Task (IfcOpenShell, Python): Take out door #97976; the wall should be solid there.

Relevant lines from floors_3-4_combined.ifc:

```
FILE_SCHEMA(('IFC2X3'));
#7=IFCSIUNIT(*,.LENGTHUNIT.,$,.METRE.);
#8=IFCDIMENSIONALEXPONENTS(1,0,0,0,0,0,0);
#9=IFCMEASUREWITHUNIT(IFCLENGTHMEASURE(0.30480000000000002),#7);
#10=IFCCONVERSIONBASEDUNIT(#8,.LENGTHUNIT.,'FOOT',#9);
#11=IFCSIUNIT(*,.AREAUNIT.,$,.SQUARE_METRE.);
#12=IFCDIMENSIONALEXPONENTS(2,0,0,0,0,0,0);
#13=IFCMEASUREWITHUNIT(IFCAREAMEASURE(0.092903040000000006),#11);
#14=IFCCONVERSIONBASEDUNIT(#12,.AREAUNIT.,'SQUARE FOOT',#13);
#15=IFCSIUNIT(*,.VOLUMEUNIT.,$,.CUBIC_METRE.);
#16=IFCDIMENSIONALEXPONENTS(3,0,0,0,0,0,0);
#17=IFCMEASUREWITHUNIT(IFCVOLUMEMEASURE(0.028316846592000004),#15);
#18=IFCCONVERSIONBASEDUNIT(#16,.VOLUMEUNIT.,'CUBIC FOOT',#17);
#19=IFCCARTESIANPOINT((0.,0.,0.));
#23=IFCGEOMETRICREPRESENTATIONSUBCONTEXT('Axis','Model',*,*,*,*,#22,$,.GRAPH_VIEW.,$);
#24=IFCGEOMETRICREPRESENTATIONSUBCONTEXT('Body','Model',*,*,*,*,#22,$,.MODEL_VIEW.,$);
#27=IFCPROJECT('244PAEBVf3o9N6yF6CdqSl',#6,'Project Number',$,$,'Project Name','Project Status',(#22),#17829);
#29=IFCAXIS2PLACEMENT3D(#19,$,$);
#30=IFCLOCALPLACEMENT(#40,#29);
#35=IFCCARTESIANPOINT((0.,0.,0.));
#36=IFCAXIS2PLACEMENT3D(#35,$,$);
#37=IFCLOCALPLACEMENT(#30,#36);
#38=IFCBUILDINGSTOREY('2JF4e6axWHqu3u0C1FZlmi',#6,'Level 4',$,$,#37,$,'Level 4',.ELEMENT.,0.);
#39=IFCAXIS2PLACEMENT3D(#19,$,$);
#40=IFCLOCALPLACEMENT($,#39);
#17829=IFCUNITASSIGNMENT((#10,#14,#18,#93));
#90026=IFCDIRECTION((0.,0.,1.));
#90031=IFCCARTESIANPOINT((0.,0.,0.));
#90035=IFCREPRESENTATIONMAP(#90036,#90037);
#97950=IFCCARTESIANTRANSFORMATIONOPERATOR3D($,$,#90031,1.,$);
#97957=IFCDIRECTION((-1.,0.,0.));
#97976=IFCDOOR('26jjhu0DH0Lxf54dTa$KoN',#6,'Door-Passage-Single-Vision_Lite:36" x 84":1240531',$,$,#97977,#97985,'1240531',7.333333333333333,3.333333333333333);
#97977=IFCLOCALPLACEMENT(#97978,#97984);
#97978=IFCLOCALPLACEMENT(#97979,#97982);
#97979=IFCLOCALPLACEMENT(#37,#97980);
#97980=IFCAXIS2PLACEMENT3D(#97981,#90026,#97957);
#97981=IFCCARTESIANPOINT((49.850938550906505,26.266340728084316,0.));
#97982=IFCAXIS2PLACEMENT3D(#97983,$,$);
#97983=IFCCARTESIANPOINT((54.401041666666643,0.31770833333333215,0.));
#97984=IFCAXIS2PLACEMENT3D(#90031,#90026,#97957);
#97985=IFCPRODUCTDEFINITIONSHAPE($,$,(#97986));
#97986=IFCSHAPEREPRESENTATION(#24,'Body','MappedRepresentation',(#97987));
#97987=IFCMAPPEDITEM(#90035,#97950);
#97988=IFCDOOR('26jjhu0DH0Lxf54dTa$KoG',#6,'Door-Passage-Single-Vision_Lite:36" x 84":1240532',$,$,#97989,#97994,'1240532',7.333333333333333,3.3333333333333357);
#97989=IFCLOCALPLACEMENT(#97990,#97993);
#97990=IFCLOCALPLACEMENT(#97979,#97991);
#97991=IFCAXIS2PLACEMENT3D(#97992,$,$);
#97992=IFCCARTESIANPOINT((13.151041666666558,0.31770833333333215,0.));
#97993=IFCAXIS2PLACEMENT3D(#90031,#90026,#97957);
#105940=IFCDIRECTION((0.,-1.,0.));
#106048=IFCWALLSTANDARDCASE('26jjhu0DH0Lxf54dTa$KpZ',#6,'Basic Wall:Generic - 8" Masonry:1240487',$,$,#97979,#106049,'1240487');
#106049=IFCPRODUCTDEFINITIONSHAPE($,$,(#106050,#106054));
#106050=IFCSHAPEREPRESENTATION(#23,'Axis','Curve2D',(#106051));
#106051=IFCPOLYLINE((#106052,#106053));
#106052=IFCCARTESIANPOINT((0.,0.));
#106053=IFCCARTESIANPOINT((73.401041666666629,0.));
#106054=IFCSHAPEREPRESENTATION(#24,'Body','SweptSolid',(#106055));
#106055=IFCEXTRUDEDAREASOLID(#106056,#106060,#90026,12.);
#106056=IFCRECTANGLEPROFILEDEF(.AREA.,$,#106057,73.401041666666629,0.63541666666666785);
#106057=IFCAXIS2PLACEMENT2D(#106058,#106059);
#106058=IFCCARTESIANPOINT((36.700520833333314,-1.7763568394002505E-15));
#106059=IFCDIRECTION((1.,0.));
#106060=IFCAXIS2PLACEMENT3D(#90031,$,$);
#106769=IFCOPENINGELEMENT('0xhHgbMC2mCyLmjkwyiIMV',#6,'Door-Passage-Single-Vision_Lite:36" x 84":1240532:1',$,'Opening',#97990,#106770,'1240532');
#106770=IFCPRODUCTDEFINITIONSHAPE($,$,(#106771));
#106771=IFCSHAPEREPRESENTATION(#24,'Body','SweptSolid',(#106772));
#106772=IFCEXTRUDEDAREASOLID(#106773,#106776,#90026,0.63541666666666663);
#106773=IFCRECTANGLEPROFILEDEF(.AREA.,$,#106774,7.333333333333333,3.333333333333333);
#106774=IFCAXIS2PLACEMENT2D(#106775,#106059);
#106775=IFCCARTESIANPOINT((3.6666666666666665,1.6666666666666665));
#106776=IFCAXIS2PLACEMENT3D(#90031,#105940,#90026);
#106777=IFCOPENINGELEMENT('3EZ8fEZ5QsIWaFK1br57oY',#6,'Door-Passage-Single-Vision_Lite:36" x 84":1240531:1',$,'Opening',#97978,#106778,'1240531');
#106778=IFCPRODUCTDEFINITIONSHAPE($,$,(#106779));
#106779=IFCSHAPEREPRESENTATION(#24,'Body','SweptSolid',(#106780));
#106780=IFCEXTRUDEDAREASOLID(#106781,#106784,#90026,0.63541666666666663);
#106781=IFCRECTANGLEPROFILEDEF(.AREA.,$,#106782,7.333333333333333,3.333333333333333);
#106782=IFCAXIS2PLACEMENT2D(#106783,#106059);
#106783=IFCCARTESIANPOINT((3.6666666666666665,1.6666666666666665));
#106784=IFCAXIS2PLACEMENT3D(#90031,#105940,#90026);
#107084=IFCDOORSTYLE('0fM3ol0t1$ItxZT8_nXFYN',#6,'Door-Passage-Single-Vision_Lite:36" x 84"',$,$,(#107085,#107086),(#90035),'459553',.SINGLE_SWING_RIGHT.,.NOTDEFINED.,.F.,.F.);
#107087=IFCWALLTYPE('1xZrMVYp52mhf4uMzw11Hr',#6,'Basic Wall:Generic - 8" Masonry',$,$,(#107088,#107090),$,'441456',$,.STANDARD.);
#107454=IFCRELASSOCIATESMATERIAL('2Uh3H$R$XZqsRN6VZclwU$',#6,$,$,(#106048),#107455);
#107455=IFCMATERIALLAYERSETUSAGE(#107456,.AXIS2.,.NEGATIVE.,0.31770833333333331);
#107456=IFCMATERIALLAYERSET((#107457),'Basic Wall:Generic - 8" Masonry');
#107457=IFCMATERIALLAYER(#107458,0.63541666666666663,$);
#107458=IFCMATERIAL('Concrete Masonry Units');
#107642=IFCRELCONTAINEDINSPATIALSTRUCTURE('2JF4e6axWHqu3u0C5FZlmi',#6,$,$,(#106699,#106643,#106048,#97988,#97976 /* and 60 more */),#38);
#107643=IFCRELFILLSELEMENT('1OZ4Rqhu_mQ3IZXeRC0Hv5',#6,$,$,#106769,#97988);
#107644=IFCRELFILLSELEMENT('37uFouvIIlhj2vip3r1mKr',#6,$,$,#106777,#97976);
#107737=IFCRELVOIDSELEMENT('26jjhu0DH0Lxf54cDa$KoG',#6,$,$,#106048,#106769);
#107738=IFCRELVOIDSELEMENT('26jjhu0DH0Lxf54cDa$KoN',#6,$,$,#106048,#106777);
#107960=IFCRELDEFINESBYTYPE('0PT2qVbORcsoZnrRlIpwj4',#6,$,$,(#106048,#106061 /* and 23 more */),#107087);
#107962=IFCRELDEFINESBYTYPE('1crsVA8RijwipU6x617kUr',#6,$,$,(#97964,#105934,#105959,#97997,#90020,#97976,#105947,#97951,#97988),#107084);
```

```python
import ifcopenshell
import ifcopenshell.api.feature
import ifcopenshell.api.root
import ifcopenshell.geom
import ifcopenshell.util.shape

model = ifcopenshell.open("floors_3-4_combined.ifc")
settings = ifcopenshell.geom.settings()


def volume(element):
    """Net volume in cubic metres, openings subtracted."""
    shape = ifcopenshell.geom.create_shape(settings, element)
    return ifcopenshell.util.shape.get_volume(shape.geometry)


door = model.by_guid("26jjhu0DH0Lxf54dTa$KoN")
opening = door.FillsVoids[0].RelatingOpeningElement
wall = opening.VoidsElements[0].RelatingBuildingElement
before = volume(wall)

ifcopenshell.api.root.remove_product(model, product=door)
ifcopenshell.api.feature.remove_feature(model, feature=opening)

after = volume(wall)

print(f"wall volume {before:.3f} -> {after:.3f} m3")

model.write("floors_3-4_combined-out.ifc")
```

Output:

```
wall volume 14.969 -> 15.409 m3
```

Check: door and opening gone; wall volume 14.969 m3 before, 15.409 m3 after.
